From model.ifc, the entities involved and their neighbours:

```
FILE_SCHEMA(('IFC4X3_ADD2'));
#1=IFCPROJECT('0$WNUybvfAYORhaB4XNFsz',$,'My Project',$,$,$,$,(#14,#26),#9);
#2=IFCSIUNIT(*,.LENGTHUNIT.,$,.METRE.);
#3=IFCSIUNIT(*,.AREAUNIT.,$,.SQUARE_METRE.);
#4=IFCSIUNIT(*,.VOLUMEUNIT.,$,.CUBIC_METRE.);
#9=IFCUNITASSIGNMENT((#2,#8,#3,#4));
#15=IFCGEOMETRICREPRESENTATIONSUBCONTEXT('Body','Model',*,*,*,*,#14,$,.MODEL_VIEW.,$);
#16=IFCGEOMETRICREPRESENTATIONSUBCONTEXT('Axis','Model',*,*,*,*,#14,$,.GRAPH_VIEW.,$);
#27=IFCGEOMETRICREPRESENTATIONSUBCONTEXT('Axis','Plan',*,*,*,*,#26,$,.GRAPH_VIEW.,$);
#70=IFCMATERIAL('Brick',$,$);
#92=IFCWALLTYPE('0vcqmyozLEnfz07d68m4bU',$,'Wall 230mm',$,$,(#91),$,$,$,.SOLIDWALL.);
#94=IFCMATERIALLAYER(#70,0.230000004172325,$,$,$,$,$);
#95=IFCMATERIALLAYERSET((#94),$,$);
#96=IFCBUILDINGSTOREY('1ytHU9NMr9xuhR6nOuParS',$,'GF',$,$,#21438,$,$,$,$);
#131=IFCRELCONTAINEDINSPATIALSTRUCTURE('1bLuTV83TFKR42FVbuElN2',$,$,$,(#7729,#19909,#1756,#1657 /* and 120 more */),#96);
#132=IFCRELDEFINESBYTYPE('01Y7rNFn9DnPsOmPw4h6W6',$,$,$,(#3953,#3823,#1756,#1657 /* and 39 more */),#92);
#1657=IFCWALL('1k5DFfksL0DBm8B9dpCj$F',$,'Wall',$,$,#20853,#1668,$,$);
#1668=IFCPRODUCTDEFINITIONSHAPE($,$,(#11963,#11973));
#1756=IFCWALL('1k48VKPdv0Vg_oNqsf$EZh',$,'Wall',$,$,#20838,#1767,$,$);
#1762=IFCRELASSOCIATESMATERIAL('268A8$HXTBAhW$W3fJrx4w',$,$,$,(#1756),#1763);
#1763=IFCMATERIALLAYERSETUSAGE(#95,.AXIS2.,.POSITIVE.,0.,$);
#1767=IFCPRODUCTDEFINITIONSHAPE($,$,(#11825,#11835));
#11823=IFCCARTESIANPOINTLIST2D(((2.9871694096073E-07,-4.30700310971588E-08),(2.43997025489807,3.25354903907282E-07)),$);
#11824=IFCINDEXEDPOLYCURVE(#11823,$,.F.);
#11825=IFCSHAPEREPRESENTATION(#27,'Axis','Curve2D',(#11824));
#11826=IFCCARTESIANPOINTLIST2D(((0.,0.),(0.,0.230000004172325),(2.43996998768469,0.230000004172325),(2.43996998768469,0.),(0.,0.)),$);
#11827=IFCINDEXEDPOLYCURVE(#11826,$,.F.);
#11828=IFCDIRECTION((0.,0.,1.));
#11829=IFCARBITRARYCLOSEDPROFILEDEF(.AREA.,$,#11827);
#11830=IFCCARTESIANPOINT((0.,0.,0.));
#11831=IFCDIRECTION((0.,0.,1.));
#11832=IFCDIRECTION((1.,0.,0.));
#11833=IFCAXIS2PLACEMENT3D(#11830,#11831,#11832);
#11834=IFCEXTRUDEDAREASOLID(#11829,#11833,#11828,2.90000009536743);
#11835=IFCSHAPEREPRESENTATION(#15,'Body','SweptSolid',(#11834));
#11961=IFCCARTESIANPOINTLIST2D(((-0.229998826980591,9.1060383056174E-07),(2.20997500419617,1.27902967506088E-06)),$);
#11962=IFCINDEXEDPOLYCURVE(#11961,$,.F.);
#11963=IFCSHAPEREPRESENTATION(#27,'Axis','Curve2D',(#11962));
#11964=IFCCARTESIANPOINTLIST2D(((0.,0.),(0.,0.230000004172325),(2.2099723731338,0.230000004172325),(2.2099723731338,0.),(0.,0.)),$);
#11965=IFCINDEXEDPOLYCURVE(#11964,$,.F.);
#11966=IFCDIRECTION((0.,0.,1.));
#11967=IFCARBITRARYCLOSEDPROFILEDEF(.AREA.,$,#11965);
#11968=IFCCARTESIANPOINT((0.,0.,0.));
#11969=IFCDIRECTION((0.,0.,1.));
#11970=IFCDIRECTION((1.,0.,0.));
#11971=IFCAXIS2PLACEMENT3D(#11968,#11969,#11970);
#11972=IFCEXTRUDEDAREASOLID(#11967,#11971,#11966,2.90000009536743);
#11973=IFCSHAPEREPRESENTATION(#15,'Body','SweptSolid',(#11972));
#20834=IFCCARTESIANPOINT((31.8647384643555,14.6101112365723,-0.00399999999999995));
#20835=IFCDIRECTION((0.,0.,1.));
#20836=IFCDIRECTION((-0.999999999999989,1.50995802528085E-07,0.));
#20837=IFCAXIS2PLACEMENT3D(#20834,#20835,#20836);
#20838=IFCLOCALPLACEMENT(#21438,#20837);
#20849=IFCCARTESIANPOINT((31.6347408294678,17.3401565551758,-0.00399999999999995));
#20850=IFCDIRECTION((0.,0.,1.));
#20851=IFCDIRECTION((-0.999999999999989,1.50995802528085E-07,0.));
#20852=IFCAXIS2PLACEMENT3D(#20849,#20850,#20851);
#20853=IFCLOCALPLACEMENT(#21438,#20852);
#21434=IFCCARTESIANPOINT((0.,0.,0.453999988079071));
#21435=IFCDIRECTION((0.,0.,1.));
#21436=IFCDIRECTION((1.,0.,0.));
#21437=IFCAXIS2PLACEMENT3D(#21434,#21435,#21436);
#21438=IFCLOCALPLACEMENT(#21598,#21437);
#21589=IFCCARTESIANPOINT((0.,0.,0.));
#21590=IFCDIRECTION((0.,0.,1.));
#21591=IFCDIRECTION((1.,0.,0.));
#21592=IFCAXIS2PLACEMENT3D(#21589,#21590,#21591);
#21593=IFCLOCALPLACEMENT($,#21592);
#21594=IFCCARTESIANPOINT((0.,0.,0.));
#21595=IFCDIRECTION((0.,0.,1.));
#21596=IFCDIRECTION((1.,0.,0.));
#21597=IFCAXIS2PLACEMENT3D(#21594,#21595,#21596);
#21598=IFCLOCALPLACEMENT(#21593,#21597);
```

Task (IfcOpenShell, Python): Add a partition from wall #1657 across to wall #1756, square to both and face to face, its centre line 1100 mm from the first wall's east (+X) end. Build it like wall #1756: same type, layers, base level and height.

```python
import numpy as np
import ifcopenshell
import ifcopenshell.api.geometry
import ifcopenshell.api.material
import ifcopenshell.api.pset
import ifcopenshell.api.root
import ifcopenshell.api.spatial
import ifcopenshell.api.type
import ifcopenshell.geom
import ifcopenshell.util.element
import ifcopenshell.util.placement
import ifcopenshell.util.representation
import ifcopenshell.util.shape
import ifcopenshell.util.unit

model = ifcopenshell.open("model.ifc")
unit_scale = ifcopenshell.util.unit.calculate_unit_scale(model)
settings = ifcopenshell.geom.settings()
settings.set("use-world-coords", True)

start_wall = model.by_guid("1k5DFfksL0DBm8B9dpCj$F")
end_wall = model.by_id(1756)
like = model.by_guid("1k48VKPdv0Vg_oNqsf$EZh")
matrix = ifcopenshell.util.placement.get_local_placement(start_wall.ObjectPlacement)
matrix[:3, 3] *= unit_scale


def extent(element):
    """Bounding box in the first wall's axes, in metres."""
    shape = ifcopenshell.geom.create_shape(settings, element)
    points = (ifcopenshell.util.shape.get_vertices(shape.geometry) - matrix[:3, 3]) @ matrix[:3, :3]
    return points.min(axis=0), points.max(axis=0)


y_start = extent(start_wall)[1][1]
y_end = extent(end_wall)[0][1]
like_min, like_max = extent(like)
length, height = float(abs(y_end - y_start)), float(like_max[2] - like_min[2])
layer_set = ifcopenshell.util.element.get_material(like, should_skip_usage=True)
thickness = sum(layer.LayerThickness for layer in layer_set.MaterialLayers) * unit_scale

wall = ifcopenshell.api.root.create_entity(model, ifc_class="IfcWall", name="New partition")
storey = ifcopenshell.util.element.get_container(like)
ifcopenshell.api.spatial.assign_container(model, products=[wall], relating_structure=storey)
ifcopenshell.api.type.assign_type(
    model, related_objects=[wall], relating_type=ifcopenshell.util.element.get_type(like), should_map_representations=False
)
rel = ifcopenshell.api.material.assign_material(
    model, products=[wall], type="IfcMaterialLayerSetUsage", material=layer_set
)
rel.RelatingMaterial.OffsetFromReferenceLine = -thickness / 2 / unit_scale
pset = ifcopenshell.api.pset.add_pset(model, product=wall, name="Pset_WallCommon")
ifcopenshell.api.pset.edit_pset(model, pset=pset, properties={"IsExternal": False, "LoadBearing": False})

# The axis runs down the middle of the wall.
axis = ifcopenshell.api.geometry.add_axis_representation(
    model, context=ifcopenshell.util.representation.get_context(model, "Model", "Axis"), axis=[(0.0, 0.0), (length, 0.0)]
)
body = ifcopenshell.api.geometry.add_wall_representation(
    model,
    context=ifcopenshell.util.representation.get_context(model, "Model", "Body", "MODEL_VIEW"),
    length=length,
    height=height,
    thickness=thickness,
    offset=-thickness / 2,
)
for representation in (axis, body):
    ifcopenshell.api.geometry.assign_representation(model, product=wall, representation=representation)

placement = matrix @ ifcopenshell.util.placement.rotation(90, "Z")
placement[:, 3] = matrix @ np.array([extent(start_wall)[0][0] + 1.1, y_start, like_min[2], 1.0])
ifcopenshell.api.geometry.edit_object_placement(model, product=wall, matrix=placement)

print(f"partition {length:.3f} m long, {height:.3f} m high, {thickness:.3f} m thick")

model.write("model-out.ifc")
```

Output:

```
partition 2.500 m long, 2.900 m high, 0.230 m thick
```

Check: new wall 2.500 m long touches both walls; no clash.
